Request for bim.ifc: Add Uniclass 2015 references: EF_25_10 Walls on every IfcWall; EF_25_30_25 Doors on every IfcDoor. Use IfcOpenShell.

First a look at what the model holds.

```python
import ifcopenshell

model = ifcopenshell.open("bim.ifc")
print(model.schema)
print("classifications:", [c.Name for c in model.by_type("IfcClassification")])
for ifc_class in ("IfcDoor", "IfcRoof", "IfcStair", "IfcWall", "IfcWindow"):
    print(ifc_class, len(model.by_type(ifc_class)))
```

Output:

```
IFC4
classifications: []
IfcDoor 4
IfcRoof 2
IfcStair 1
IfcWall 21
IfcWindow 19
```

```python
import ifcopenshell
import ifcopenshell.api.classification

model = ifcopenshell.open("bim.ifc")

system = ifcopenshell.api.classification.add_classification(model, classification="Uniclass 2015")

codes = {
    "IfcWall": ("EF_25_10", "Walls"),
    "IfcDoor": ("EF_25_30_25", "Doors"),
}
for ifc_class, (code, name) in codes.items():
    products = model.by_type(ifc_class)
    ifcopenshell.api.classification.add_reference(
        model, products=products, classification=system, identification=code, name=name
    )
    print(code, len(products))

model.write("bim_v2.ifc")
```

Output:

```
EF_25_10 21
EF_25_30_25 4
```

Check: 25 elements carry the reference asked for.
